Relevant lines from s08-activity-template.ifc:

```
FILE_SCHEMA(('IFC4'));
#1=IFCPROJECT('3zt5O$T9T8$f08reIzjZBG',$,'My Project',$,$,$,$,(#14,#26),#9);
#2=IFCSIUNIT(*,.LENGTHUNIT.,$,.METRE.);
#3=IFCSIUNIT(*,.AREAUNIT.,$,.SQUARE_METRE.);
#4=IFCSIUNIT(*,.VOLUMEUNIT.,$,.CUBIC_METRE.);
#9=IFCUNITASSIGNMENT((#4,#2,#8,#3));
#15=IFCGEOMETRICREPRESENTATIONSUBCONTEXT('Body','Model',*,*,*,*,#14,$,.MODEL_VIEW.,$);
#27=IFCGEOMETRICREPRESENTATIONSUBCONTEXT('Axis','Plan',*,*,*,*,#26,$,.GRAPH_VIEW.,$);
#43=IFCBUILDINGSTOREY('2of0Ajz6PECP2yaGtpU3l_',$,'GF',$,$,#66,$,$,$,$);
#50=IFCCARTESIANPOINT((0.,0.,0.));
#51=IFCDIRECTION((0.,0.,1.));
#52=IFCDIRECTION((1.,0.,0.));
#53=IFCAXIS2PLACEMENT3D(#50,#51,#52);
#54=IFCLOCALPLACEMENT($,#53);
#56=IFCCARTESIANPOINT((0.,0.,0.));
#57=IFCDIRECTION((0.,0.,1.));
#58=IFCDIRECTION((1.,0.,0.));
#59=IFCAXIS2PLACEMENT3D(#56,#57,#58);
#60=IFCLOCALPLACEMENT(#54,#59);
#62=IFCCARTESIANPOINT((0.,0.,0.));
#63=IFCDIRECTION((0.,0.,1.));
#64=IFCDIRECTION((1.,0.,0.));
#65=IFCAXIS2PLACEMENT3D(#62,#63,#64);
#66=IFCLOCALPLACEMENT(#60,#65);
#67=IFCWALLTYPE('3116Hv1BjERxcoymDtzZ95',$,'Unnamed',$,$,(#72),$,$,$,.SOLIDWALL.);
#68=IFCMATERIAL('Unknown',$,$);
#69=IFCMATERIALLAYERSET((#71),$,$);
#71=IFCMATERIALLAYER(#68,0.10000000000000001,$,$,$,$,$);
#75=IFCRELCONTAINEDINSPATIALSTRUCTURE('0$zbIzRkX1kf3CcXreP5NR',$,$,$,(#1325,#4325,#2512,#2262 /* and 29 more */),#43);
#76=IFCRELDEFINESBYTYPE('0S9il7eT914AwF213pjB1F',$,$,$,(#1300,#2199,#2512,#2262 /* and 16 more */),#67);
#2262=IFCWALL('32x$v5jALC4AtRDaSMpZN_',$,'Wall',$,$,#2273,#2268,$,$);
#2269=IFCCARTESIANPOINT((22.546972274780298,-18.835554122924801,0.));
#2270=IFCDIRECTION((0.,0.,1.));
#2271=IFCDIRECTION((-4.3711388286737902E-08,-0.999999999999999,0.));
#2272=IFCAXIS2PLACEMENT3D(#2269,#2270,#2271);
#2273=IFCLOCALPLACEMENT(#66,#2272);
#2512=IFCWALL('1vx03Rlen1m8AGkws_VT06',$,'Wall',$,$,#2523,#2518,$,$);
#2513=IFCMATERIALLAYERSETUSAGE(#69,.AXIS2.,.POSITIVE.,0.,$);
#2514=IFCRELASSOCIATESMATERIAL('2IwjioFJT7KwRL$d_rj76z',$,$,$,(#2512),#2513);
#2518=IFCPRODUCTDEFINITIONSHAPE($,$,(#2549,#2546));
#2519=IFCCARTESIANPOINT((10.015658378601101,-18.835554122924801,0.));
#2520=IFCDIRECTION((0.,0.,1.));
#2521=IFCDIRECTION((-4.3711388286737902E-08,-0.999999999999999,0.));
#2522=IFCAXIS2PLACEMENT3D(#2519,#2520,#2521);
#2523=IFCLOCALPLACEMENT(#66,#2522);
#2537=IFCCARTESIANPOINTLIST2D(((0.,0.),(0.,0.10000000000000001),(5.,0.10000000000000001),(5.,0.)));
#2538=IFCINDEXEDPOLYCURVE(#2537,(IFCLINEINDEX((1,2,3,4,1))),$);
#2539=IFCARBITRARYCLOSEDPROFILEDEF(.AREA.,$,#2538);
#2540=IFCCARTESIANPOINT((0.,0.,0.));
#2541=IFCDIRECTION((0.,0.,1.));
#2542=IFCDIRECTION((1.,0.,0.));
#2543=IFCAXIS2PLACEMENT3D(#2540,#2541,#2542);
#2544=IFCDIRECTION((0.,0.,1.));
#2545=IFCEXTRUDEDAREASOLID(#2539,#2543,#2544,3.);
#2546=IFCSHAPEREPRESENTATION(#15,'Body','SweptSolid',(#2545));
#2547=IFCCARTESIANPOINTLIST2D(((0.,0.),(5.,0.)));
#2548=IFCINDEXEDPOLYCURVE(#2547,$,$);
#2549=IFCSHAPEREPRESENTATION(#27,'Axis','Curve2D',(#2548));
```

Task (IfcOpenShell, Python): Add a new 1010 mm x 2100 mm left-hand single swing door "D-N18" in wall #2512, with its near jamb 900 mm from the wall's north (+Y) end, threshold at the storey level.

```python
import numpy as np
import ifcopenshell
import ifcopenshell.api.feature
import ifcopenshell.api.geometry
import ifcopenshell.api.root
import ifcopenshell.api.spatial
import ifcopenshell.geom
import ifcopenshell.util.element
import ifcopenshell.util.placement
import ifcopenshell.util.representation
import ifcopenshell.util.shape
import ifcopenshell.util.unit

model = ifcopenshell.open("s08-activity-template.ifc")
unit_scale = ifcopenshell.util.unit.calculate_unit_scale(model)
settings = ifcopenshell.geom.settings()


def volume(element):
    """Net volume in cubic metres, openings subtracted."""
    shape = ifcopenshell.geom.create_shape(settings, element)
    return ifcopenshell.util.shape.get_volume(shape.geometry)


wall = model.by_guid("1vx03Rlen1m8AGkws_VT06")
storey = ifcopenshell.util.element.get_container(wall, ifc_class="IfcBuildingStorey")
context = ifcopenshell.util.representation.get_context(model, "Model", "Body", "MODEL_VIEW")
before = volume(wall)

width, height, from_end, sill = 1.01, 2.1, 0.9, 0.0  # metres

# The wall runs along its own X axis, and the end named is its -X end.
wall_shape = ifcopenshell.geom.create_shape(settings, wall)
x, y, z = ifcopenshell.util.shape.get_vertices(wall_shape.geometry).T
start = x.min() + from_end
face, thickness = float(y.min()), float(y.max() - y.min())
wall_matrix = ifcopenshell.util.placement.get_local_placement(wall.ObjectPlacement)
level = ifcopenshell.util.placement.get_local_placement(storey.ObjectPlacement)[2, 3]


def in_wall(x, y):
    """Placement at x, y metres in the wall's axes, at sill height."""
    matrix = wall_matrix.copy()
    matrix[:, 3] = wall_matrix @ np.array([x / unit_scale, y / unit_scale, 0.0, 1.0])
    matrix[2, 3] = level + sill / unit_scale
    return matrix


# Opening: a box that overshoots both wall faces by 50 mm.
opening = ifcopenshell.api.root.create_entity(model, ifc_class="IfcOpeningElement", predefined_type="OPENING")
box = ifcopenshell.api.geometry.add_wall_representation(
    model, context=context, length=width, height=height, thickness=thickness + 0.1
)
ifcopenshell.api.geometry.assign_representation(model, product=opening, representation=box)
ifcopenshell.api.geometry.edit_object_placement(model, product=opening, matrix=in_wall(start, face - 0.05), is_si=False)
ifcopenshell.api.feature.add_feature(model, feature=opening, element=wall)

door = ifcopenshell.api.root.create_entity(model, ifc_class="IfcDoor", name="D-N18", predefined_type="DOOR")
door.OverallWidth, door.OverallHeight = width / unit_scale, height / unit_scale
door.OperationType = "SINGLE_SWING_LEFT"
body = ifcopenshell.api.geometry.add_door_representation(
    model,
    context=context,
    overall_width=door.OverallWidth,
    overall_height=door.OverallHeight,
    operation_type="SINGLE_SWING_LEFT",
    lining_properties={"LiningDepth": thickness / unit_scale, "ThresholdDepth": thickness / unit_scale},
)
ifcopenshell.api.geometry.assign_representation(model, product=door, representation=body)
ifcopenshell.api.spatial.assign_container(model, products=[door], relating_structure=storey)
ifcopenshell.api.feature.add_filling(model, opening=opening, element=door)

# The lining spans the wall, so the door starts at the wall face.
ifcopenshell.api.geometry.edit_object_placement(model, product=door, matrix=in_wall(start, face), is_si=False)

after = volume(wall)

print(f"wall volume {before:.3f} -> {after:.3f} m3")

model.write("s08-activity-template_updated.ifc")
```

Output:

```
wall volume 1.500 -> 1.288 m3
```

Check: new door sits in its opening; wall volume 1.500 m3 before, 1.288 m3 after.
